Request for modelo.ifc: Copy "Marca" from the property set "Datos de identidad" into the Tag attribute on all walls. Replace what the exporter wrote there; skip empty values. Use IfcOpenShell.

First a look at what the model holds.

```python
import ifcopenshell
import ifcopenshell.util.element

model = ifcopenshell.open("modelo.ifc")
print(model.schema)
walls = model.by_type("IfcWall")
print(len(walls), "walls")
for e in walls[:8]:
    source = ifcopenshell.util.element.get_pset(e, "Datos de identidad", "Marca")
    target = e.Tag
    print(e.id(), repr(source), repr(target), sep=" | ")
```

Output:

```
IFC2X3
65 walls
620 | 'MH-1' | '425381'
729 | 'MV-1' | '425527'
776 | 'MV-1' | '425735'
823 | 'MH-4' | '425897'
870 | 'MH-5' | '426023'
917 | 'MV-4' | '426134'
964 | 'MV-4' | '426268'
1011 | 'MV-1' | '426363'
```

```python
import ifcopenshell
import ifcopenshell.util.element

model = ifcopenshell.open("modelo.ifc")

count = 0
for e in model.by_type("IfcWall"):
    value = ifcopenshell.util.element.get_pset(e, "Datos de identidad", "Marca")
    current = e.Tag
    if not value or not value.strip() or current == value:
        continue
    e.Tag = value
    count += 1

print(count, "walls updated")

model.write("modelo_edited.ifc")
```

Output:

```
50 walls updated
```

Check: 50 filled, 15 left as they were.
